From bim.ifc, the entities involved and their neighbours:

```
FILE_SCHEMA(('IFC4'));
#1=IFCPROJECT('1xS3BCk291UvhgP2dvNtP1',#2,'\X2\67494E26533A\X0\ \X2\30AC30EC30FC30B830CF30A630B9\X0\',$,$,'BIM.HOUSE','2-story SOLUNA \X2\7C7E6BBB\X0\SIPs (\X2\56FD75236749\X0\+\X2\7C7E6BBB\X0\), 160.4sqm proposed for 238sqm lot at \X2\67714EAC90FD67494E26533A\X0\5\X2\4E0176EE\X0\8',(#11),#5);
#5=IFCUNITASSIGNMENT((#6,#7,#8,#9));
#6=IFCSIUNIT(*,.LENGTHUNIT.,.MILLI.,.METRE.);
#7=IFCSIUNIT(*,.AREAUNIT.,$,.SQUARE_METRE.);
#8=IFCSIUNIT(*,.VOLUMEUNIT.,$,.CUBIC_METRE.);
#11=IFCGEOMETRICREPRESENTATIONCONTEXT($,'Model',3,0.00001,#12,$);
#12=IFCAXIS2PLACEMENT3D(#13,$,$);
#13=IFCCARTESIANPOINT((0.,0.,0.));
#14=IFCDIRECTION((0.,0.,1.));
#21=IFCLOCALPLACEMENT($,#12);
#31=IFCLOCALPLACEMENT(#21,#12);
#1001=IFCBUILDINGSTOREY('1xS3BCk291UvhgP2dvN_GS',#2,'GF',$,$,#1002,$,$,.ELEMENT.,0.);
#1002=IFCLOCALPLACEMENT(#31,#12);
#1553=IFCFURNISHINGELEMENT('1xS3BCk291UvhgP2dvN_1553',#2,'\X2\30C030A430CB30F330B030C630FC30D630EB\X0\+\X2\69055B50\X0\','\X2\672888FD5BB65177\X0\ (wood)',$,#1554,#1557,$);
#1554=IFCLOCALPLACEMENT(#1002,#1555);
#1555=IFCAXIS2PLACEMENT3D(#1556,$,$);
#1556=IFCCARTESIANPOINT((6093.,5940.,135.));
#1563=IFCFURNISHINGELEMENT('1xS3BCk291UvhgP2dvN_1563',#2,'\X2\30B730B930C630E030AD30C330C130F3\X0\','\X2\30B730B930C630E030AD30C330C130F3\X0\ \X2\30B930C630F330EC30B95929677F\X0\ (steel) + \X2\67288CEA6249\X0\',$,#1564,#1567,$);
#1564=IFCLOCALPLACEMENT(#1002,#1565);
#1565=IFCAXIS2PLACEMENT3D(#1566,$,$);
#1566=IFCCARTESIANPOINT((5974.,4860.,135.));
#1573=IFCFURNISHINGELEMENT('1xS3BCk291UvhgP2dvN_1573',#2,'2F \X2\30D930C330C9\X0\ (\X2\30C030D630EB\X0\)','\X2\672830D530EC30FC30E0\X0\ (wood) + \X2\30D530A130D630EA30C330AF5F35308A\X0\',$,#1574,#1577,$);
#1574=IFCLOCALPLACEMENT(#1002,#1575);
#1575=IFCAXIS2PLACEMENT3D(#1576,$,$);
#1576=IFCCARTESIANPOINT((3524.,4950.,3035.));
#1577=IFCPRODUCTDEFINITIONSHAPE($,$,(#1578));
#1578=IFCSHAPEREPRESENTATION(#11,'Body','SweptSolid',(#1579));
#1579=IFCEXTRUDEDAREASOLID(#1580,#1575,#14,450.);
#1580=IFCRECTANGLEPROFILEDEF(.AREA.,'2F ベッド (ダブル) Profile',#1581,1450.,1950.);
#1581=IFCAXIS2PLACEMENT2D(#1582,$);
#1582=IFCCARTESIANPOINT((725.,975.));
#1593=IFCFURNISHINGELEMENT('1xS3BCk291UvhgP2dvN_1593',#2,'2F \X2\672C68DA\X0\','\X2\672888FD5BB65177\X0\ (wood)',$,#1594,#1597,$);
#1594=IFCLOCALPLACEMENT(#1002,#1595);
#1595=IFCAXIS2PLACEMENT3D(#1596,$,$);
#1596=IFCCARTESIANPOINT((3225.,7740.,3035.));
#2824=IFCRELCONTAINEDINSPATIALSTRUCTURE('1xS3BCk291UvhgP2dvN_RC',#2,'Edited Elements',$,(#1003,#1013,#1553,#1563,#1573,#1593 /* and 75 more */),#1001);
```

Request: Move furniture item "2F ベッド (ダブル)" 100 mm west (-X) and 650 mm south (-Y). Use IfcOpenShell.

```python
import ifcopenshell
import ifcopenshell.api.geometry
import ifcopenshell.util.placement
import ifcopenshell.util.unit

model = ifcopenshell.open("bim.ifc")
unit_scale = ifcopenshell.util.unit.calculate_unit_scale(model)

item = model.by_id(1573)
matrix = ifcopenshell.util.placement.get_local_placement(item.ObjectPlacement)
matrix[0, 3] -= 0.1 / unit_scale
matrix[1, 3] -= 0.65 / unit_scale
ifcopenshell.api.geometry.edit_object_placement(model, product=item, matrix=matrix, is_si=False)

print(ifcopenshell.util.placement.get_local_placement(item.ObjectPlacement).round(3) + 0.0)

model.write("bim-out.ifc")
```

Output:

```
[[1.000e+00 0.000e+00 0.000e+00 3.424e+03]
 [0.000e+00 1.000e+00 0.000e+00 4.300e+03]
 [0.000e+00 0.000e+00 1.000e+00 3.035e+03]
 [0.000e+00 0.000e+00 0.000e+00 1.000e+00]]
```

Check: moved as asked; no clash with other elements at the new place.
